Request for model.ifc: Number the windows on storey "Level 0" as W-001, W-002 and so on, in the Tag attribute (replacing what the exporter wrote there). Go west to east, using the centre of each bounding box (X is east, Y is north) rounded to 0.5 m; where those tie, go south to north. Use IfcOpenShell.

First a look at what the model holds.

```python
import ifcopenshell
import ifcopenshell.util.element
import ifcopenshell.util.placement

model = ifcopenshell.open("model.ifc")
print(model.schema)
storey = next(s for s in model.by_type("IfcBuildingStorey") if s.Name == "Level 0")
windows = [e for e in ifcopenshell.util.element.get_decomposition(storey) if e.is_a("IfcWindow")]
for e in sorted(windows, key=lambda e: e.id()):
    origin = ifcopenshell.util.placement.get_local_placement(e.ObjectPlacement)[:3, 3]
    print(e.id(), e.Tag, e.Name, origin.round(2) + 0.0, sep=" | ")
```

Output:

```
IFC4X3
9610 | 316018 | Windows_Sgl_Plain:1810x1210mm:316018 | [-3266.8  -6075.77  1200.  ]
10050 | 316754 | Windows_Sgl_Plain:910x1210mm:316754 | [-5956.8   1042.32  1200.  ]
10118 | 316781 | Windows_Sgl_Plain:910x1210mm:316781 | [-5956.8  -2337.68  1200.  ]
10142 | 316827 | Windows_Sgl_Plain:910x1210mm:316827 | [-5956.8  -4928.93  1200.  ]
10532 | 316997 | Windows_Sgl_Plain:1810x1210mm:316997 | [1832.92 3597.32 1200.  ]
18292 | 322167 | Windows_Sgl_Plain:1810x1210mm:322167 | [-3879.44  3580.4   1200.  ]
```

```python
import ifcopenshell
import ifcopenshell.geom
import ifcopenshell.util.element
import ifcopenshell.util.shape

model = ifcopenshell.open("model.ifc")
settings = ifcopenshell.geom.settings()
settings.set("use-world-coords", True)


def centre(element):
    shape = ifcopenshell.geom.create_shape(settings, element)
    return ifcopenshell.util.shape.get_bbox_centroid(shape.geometry)


storey = next(s for s in model.by_type("IfcBuildingStorey") if s.Name == "Level 0")
windows = [e for e in ifcopenshell.util.element.get_decomposition(storey) if e.is_a("IfcWindow")]

# Insertion points can sit at a corner or the storey origin, so sort by the geometry (in metres).
centres = {e: centre(e) for e in windows}
windows.sort(key=lambda e: (round(centres[e][0] / 0.5), centres[e][1]))

for i, e in enumerate(windows, start=1):
    number = f"W-0{i:02d}"
    e.Tag = number
    print(e.id(), number)

model.write("model_v2.ifc")
```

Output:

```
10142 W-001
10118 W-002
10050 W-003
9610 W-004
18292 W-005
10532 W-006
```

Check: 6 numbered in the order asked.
